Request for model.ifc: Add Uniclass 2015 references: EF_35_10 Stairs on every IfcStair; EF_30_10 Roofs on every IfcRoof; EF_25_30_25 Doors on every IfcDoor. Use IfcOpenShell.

First a look at what the model holds.

```python
import ifcopenshell

model = ifcopenshell.open("model.ifc")
print(model.schema)
print("classifications:", [c.Name for c in model.by_type("IfcClassification")])
for ifc_class in ("IfcDoor", "IfcRoof", "IfcStair", "IfcWall", "IfcWindow"):
    print(ifc_class, len(model.by_type(ifc_class)))
```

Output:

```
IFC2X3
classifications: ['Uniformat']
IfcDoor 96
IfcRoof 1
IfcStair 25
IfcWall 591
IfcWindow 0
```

```python
import ifcopenshell
import ifcopenshell.api.classification

model = ifcopenshell.open("model.ifc")

# IFC2X3 requires Source and Edition and has no link from the project to the system.
system = model.create_entity("IfcClassification", Source="NBS", Edition="2015", Name="Uniclass 2015")

codes = {
    "IfcStair": ("EF_35_10", "Stairs"),
    "IfcRoof": ("EF_30_10", "Roofs"),
    "IfcDoor": ("EF_25_30_25", "Doors"),
}
for ifc_class, (code, name) in codes.items():
    products = model.by_type(ifc_class)
    ifcopenshell.api.classification.add_reference(
        model, products=products, classification=system, identification=code, name=name
    )
    print(code, len(products))

model.write("model_updated.ifc")
```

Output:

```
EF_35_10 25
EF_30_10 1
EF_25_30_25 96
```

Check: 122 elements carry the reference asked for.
